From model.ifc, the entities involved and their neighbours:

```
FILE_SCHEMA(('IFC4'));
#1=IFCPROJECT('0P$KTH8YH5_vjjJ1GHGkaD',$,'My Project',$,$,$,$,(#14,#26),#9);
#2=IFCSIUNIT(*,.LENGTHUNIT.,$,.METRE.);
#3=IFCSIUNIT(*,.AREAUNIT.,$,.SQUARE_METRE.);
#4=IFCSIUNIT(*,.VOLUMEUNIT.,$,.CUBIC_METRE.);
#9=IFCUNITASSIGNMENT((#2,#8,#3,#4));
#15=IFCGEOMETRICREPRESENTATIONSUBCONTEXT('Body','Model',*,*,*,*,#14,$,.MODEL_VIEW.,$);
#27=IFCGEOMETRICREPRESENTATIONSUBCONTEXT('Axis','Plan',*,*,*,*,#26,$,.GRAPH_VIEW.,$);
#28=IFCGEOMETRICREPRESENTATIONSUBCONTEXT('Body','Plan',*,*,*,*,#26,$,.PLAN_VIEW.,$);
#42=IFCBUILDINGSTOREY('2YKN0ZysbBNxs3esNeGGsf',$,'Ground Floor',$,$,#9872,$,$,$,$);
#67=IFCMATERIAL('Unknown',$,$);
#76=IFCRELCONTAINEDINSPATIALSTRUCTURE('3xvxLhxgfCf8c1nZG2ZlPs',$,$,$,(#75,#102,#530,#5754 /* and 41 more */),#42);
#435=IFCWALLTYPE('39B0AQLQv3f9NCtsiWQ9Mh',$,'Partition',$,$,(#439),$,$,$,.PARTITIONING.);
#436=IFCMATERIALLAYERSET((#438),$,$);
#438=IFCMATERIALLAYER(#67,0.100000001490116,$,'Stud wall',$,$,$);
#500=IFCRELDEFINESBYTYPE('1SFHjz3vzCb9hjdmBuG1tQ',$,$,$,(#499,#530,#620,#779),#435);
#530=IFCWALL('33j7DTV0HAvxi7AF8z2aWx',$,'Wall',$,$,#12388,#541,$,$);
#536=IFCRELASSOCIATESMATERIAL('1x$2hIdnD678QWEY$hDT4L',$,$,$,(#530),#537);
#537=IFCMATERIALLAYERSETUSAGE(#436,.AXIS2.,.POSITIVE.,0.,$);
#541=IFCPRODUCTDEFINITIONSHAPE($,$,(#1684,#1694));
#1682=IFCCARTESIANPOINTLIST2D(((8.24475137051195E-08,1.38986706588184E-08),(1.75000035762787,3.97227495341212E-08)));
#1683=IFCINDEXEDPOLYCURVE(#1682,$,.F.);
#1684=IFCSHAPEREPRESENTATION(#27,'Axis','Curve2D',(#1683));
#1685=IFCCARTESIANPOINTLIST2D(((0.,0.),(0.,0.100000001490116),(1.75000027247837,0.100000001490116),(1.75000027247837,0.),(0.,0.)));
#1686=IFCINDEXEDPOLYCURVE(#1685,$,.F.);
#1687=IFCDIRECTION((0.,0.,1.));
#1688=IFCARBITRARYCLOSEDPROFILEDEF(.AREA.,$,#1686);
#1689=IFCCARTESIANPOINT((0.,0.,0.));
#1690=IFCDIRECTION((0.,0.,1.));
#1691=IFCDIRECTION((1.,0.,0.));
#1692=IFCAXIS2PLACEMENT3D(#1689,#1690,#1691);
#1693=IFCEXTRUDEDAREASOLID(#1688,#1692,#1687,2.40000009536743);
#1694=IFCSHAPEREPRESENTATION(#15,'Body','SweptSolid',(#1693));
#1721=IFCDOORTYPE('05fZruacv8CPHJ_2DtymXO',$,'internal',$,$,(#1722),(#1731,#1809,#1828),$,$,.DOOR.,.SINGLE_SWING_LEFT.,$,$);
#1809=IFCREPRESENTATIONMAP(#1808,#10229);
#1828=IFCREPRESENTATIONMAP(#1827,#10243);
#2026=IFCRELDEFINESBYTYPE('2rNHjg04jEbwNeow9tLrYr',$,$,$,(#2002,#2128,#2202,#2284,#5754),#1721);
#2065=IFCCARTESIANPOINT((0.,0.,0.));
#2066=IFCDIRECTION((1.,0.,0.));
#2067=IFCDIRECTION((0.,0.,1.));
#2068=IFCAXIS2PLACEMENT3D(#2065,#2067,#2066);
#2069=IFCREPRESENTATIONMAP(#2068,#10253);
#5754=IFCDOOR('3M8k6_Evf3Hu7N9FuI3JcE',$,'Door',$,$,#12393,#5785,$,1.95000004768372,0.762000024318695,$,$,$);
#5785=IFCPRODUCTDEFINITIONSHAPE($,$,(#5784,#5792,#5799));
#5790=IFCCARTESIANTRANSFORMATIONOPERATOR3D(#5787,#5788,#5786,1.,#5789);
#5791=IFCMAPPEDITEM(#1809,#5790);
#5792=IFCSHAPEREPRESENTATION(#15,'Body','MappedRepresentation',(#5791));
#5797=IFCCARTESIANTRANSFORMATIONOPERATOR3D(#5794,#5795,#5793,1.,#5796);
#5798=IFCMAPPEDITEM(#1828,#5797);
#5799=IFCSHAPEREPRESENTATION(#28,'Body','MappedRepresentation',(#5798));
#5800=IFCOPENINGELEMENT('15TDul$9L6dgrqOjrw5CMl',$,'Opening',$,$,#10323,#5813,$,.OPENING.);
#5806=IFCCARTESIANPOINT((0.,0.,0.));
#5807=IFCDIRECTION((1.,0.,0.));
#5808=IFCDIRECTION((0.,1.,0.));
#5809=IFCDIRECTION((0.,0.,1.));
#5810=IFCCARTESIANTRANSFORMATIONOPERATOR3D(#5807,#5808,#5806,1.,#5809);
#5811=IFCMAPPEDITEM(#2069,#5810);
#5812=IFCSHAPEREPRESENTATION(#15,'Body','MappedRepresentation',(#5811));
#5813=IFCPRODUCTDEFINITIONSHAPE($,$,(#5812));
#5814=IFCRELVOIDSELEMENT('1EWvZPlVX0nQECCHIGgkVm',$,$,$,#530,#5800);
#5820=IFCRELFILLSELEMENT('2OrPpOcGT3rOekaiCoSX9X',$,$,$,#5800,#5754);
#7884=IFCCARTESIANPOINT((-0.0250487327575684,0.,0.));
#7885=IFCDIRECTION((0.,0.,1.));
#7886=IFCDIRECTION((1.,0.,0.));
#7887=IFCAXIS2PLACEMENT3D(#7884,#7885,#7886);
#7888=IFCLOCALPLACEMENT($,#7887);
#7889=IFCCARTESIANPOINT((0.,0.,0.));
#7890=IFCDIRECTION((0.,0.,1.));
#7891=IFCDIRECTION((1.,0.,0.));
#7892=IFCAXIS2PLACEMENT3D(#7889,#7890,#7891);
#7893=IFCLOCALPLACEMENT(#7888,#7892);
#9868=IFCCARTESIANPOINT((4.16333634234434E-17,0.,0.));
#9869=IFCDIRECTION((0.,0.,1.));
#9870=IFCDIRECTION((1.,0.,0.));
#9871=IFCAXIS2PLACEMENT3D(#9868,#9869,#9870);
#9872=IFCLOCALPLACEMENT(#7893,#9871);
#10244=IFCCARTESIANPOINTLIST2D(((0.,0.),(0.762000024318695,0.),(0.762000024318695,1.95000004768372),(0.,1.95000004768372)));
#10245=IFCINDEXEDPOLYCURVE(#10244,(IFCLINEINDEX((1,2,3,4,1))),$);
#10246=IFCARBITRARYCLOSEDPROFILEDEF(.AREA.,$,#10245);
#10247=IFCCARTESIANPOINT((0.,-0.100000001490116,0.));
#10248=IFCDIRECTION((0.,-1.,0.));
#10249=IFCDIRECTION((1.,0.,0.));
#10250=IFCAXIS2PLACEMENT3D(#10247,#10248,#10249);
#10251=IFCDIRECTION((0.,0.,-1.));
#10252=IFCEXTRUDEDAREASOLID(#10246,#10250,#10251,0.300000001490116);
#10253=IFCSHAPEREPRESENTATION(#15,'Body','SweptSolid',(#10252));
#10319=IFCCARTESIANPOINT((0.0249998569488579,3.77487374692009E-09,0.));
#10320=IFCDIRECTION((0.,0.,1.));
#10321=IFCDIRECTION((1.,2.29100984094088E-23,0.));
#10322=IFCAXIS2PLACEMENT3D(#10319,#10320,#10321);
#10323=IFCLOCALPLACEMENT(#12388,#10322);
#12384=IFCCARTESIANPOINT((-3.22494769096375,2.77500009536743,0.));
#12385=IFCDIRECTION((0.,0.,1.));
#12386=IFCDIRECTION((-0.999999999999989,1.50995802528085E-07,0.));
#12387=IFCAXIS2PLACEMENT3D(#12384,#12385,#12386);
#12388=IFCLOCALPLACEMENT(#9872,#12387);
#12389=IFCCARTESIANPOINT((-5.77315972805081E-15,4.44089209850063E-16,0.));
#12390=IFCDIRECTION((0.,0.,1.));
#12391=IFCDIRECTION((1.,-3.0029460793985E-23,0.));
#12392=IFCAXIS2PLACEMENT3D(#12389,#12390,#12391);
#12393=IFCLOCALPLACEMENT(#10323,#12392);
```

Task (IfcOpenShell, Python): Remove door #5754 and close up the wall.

```python
import ifcopenshell
import ifcopenshell.api.feature
import ifcopenshell.api.root
import ifcopenshell.geom
import ifcopenshell.util.shape

model = ifcopenshell.open("model.ifc")
settings = ifcopenshell.geom.settings()


def volume(element):
    """Net volume in cubic metres, openings subtracted."""
    shape = ifcopenshell.geom.create_shape(settings, element)
    return ifcopenshell.util.shape.get_volume(shape.geometry)


door = model.by_id(5754)
opening = door.FillsVoids[0].RelatingOpeningElement
wall = opening.VoidsElements[0].RelatingBuildingElement
before = volume(wall)

ifcopenshell.api.root.remove_product(model, product=door)
ifcopenshell.api.feature.remove_feature(model, feature=opening)

after = volume(wall)

print(f"wall volume {before:.3f} -> {after:.3f} m3")

model.write("model_edited.ifc")
```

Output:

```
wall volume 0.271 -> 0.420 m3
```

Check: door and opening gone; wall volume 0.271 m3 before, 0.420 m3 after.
